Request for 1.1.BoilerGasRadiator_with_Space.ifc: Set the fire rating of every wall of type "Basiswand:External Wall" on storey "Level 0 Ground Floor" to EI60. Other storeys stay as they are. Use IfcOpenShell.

First a look at what the model holds.

```python
import ifcopenshell
import ifcopenshell.util.element

model = ifcopenshell.open("1.1.BoilerGasRadiator_with_Space.ifc")
print(model.schema)
storey = next(s for s in model.by_type("IfcBuildingStorey") if s.Name == "Level 0 Ground Floor")
walls = [e for e in ifcopenshell.util.element.get_decomposition(storey) if e.is_a("IfcWall")]
seen = {}
for e in walls:
    element_type = ifcopenshell.util.element.get_type(e)
    key = (element_type.Name if element_type != e and element_type else None, ifcopenshell.util.element.get_pset(e, "Pset_WallCommon", "FireRating"))
    seen[key] = seen.get(key, 0) + 1
for (name, value), count in sorted(seen.items(), key=str):
    print(count, "x", name, "|", value)
```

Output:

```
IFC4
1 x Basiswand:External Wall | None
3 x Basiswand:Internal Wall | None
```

```python
import ifcopenshell
import ifcopenshell.api.pset
import ifcopenshell.util.element

model = ifcopenshell.open("1.1.BoilerGasRadiator_with_Space.ifc")

storey = next(s for s in model.by_type("IfcBuildingStorey") if s.Name == "Level 0 Ground Floor")
walls = [e for e in ifcopenshell.util.element.get_decomposition(storey) if e.is_a("IfcWall")]

count = 0
for e in walls:
    element_type = ifcopenshell.util.element.get_type(e)
    if element_type in (None, e) or element_type.Name != "Basiswand:External Wall":
        continue
    # add_pset returns the element's existing set when there is one.
    pset = ifcopenshell.api.pset.add_pset(model, product=e, name="Pset_WallCommon")
    ifcopenshell.api.pset.edit_pset(model, pset=pset, properties={"FireRating": "EI60"})
    count += 1

print(count, "walls updated")

model.write("1.1.BoilerGasRadiator_with_Space-out.ifc")
```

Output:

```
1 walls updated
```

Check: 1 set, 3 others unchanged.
